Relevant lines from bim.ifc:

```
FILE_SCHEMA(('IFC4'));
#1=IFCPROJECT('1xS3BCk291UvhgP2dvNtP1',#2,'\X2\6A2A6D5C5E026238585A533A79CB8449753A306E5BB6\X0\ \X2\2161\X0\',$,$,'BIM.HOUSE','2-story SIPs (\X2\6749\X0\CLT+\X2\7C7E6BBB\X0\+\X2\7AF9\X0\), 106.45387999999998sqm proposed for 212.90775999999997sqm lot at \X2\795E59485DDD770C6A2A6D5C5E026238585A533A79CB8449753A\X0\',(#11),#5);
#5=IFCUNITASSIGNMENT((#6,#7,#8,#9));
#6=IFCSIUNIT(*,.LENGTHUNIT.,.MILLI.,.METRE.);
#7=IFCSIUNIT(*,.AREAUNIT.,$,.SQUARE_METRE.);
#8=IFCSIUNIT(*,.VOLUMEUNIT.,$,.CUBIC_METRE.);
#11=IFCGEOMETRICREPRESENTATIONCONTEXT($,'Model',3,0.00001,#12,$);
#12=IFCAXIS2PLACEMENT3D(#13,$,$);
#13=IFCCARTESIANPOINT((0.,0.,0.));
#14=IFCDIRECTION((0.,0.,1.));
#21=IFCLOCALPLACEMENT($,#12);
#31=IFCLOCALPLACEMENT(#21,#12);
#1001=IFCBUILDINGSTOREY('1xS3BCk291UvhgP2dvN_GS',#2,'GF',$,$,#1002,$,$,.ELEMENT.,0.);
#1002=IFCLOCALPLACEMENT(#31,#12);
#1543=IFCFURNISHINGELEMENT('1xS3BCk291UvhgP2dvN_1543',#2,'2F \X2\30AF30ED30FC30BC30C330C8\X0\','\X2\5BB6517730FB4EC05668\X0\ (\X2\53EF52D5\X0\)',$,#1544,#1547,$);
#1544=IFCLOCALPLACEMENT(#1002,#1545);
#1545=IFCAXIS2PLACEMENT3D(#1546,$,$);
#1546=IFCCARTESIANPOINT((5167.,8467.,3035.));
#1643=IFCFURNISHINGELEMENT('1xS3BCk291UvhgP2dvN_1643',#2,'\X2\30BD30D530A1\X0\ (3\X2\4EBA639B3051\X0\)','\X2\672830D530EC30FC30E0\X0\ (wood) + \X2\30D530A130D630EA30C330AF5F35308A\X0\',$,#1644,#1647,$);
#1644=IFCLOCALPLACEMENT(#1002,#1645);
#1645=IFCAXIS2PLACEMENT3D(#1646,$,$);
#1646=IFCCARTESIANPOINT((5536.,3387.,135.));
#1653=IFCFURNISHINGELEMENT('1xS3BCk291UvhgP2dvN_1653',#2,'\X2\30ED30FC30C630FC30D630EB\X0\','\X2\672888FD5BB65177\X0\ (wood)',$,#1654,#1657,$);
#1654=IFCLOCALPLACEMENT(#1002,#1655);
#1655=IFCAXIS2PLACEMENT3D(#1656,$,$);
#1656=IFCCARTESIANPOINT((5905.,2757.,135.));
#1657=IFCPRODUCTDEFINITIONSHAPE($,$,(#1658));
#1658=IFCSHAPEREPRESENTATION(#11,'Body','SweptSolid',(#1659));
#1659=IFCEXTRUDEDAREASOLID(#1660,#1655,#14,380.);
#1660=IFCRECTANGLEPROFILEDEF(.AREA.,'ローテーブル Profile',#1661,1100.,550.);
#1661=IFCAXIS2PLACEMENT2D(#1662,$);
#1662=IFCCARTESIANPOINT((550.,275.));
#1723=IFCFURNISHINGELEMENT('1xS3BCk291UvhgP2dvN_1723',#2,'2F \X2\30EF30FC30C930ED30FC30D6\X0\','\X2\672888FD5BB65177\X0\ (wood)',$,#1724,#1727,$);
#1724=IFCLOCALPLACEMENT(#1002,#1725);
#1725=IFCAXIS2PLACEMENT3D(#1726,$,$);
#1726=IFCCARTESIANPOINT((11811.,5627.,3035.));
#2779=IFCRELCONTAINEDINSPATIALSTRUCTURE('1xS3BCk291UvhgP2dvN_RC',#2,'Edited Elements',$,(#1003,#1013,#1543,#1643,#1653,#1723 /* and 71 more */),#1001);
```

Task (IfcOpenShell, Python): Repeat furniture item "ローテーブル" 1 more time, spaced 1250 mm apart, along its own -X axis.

```python
import ifcopenshell
import ifcopenshell.api.geometry
import ifcopenshell.api.root
import ifcopenshell.util.element
import ifcopenshell.util.placement

model = ifcopenshell.open("bim.ifc")


def reuse_history(source, copy):
    """copy_class also copies each property set's owner history, people and application; keep the originals."""
    for rel in copy.IsDefinedBy:
        if rel.is_a("IfcRelDefinesByProperties") and (history := rel.RelatingPropertyDefinition.OwnerHistory):
            rel.RelatingPropertyDefinition.OwnerHistory = source.OwnerHistory
            ifcopenshell.util.element.remove_deep2(model, history)


source = model.by_guid("1xS3BCk291UvhgP2dvN_1653")
base = ifcopenshell.util.placement.get_local_placement(source.ObjectPlacement)
step = -base[:3, 0] * 1250.0

for i in range(1, 2):
    copy = ifcopenshell.api.root.copy_class(model, product=source)
    copy.Representation = ifcopenshell.util.element.copy_deep(
        model, source.Representation, exclude=["IfcGeometricRepresentationContext", "IfcRepresentationMap"]
    )
    reuse_history(source, copy)
    matrix = base.copy()
    matrix[:3, 3] += i * step
    print("added at", matrix[:3, 3].round(3) + 0.0)
    ifcopenshell.api.geometry.edit_object_placement(model, product=copy, matrix=matrix, is_si=False)

model.write("bim_edited.ifc")
```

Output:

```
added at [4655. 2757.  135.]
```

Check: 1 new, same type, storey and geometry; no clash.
